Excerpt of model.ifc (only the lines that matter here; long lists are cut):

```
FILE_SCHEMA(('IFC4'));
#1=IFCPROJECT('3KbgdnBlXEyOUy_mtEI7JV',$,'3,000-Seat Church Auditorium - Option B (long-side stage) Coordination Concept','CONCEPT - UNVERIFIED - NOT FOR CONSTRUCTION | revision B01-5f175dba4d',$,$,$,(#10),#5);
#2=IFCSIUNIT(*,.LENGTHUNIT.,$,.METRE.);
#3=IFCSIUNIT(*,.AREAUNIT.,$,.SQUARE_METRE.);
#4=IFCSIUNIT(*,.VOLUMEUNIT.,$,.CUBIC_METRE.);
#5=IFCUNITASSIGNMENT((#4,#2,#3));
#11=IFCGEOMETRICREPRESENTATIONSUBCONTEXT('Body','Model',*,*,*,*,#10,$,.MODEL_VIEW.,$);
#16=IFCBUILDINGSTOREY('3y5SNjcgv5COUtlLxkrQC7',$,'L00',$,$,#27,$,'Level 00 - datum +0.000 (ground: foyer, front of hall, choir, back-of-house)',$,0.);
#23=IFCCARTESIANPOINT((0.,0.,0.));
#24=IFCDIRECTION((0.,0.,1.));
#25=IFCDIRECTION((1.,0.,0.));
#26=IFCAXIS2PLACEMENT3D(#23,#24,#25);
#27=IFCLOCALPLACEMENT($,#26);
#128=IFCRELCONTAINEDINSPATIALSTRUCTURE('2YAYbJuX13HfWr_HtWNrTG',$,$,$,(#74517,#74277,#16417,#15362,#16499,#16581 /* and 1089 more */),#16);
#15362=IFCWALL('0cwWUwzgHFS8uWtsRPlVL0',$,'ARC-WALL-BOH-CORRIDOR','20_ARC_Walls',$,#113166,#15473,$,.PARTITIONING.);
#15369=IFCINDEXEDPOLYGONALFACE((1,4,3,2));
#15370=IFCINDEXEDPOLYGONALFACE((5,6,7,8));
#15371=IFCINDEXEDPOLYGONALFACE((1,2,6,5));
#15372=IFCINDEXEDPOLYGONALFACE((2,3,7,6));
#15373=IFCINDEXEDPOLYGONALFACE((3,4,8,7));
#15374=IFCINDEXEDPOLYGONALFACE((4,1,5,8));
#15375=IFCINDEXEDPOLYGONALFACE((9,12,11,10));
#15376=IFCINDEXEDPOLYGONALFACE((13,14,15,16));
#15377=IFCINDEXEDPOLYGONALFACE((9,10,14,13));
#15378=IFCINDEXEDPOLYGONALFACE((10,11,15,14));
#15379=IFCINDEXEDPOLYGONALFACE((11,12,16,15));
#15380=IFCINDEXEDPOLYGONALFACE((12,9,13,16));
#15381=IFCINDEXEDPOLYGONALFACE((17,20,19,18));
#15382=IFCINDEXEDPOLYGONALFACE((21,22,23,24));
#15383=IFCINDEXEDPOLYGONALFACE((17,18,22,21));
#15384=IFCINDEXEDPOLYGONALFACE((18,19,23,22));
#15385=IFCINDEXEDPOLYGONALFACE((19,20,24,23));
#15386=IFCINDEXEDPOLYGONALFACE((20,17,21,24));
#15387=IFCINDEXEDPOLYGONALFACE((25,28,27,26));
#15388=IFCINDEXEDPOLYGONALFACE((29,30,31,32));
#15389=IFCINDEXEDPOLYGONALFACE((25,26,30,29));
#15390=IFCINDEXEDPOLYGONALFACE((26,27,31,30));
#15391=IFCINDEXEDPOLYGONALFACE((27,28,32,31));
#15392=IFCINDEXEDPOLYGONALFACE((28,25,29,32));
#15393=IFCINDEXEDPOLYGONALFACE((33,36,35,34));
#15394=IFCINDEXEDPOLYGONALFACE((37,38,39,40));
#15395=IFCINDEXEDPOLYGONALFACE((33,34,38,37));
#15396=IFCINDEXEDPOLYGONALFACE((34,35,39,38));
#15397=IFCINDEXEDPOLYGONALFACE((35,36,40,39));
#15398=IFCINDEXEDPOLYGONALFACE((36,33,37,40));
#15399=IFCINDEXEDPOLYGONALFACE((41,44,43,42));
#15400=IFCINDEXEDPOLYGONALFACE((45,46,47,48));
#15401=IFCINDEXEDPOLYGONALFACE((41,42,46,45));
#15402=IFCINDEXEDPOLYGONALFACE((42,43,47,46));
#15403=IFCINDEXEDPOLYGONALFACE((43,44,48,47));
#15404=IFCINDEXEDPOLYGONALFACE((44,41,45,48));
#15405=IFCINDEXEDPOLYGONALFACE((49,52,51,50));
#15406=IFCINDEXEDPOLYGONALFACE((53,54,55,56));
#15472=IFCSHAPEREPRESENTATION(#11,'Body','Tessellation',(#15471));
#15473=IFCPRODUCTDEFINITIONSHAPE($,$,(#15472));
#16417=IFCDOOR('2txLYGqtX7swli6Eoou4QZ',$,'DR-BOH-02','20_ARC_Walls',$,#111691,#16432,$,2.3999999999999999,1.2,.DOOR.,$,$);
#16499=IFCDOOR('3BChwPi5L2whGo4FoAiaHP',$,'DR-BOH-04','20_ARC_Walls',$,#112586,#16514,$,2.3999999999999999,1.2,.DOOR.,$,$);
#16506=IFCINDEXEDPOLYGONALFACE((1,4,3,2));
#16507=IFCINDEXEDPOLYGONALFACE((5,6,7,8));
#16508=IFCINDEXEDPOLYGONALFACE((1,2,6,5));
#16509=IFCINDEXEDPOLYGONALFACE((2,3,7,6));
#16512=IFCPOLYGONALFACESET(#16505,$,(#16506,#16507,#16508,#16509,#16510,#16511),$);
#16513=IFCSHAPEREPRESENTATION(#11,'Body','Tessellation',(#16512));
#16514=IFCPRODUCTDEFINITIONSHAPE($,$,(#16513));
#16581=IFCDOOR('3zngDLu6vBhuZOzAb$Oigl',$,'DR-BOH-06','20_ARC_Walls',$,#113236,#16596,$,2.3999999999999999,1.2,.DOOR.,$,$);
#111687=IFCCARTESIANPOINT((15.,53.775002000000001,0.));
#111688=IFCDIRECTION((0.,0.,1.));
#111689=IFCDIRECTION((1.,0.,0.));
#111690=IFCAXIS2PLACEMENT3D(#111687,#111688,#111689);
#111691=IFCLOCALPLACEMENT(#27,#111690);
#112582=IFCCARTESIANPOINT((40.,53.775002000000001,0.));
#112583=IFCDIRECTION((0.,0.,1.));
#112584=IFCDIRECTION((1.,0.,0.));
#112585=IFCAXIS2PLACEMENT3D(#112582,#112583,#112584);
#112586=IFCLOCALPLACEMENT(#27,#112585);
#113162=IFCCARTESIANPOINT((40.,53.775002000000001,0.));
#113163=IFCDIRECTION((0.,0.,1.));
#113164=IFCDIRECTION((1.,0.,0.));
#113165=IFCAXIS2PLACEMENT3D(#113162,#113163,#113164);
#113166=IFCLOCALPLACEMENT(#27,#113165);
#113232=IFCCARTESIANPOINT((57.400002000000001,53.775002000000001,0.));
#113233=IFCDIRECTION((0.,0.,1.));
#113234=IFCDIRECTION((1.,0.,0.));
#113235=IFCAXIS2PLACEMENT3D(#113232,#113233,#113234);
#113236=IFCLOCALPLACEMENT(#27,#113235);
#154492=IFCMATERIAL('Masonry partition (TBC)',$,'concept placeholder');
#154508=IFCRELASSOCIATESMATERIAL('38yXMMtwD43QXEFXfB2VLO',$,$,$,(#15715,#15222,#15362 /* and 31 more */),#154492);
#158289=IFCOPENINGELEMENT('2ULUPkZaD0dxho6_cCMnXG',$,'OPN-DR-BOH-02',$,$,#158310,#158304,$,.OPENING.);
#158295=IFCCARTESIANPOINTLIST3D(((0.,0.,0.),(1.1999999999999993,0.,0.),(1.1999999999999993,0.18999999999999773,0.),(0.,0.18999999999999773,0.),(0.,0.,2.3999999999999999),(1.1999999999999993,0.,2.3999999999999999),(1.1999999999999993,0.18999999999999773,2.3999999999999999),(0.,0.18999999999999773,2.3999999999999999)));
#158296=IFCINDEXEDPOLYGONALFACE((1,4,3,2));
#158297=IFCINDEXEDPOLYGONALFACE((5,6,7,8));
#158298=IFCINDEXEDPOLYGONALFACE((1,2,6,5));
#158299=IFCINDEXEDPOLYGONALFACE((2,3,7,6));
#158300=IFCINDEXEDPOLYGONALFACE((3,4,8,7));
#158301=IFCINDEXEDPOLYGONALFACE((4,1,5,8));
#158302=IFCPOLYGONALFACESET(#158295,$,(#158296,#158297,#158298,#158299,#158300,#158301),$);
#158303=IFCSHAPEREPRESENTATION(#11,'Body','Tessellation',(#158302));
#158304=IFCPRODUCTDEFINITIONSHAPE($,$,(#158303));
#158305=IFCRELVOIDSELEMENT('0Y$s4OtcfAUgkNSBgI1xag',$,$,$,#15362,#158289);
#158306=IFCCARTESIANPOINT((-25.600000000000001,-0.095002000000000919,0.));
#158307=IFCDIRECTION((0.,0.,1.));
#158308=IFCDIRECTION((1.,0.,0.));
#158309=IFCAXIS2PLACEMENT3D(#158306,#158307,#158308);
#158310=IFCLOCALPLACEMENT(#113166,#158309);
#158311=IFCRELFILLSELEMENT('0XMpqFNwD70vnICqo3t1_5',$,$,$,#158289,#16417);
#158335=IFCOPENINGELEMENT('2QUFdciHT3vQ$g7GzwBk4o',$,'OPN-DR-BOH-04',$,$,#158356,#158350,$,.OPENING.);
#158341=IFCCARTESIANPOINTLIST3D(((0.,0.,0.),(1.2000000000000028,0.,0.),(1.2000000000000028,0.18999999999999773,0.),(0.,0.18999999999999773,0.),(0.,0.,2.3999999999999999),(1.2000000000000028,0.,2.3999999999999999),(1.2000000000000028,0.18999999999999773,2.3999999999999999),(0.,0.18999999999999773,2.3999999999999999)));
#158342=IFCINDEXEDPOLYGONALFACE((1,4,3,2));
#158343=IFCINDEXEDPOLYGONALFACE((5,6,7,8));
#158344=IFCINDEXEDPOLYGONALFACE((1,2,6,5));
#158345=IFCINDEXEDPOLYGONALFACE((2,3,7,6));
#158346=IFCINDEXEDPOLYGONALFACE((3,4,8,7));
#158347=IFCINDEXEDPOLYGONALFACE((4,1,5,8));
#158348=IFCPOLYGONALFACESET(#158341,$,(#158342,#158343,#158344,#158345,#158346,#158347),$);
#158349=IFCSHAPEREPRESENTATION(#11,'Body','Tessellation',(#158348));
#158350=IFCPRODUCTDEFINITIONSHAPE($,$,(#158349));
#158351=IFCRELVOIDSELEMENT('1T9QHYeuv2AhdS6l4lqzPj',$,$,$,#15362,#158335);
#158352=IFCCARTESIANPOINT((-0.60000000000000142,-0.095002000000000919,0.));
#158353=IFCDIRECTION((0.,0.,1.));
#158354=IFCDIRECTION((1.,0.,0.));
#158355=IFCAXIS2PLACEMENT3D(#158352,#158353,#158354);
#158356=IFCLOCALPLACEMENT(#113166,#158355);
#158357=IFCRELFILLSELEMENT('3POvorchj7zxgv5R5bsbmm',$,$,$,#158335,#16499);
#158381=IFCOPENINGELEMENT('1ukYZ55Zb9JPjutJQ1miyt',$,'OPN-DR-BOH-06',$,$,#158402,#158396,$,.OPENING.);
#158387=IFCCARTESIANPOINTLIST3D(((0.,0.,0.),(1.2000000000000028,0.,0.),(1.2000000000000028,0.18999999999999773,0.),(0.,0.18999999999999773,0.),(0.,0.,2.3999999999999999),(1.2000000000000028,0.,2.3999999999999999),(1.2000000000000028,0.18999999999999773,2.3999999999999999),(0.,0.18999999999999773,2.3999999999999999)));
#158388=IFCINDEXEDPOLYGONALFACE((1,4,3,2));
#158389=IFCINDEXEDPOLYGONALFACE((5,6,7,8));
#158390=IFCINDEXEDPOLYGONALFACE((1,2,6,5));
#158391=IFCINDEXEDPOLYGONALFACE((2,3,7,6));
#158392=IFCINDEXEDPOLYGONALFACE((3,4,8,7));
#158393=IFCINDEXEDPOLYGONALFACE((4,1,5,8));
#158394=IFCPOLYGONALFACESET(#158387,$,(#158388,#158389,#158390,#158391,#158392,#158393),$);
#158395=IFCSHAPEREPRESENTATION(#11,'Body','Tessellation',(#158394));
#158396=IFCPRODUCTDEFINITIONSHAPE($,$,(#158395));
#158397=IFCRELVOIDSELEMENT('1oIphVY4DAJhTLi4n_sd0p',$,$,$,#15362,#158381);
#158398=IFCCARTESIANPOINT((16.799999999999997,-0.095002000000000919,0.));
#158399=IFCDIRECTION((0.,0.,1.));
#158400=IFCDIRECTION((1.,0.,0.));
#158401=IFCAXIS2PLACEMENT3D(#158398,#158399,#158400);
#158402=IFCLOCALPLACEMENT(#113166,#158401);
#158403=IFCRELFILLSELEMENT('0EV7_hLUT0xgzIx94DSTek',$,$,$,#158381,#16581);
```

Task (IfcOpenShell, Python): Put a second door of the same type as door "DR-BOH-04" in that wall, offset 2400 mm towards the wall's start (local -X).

```python
import ifcopenshell
import ifcopenshell.api.feature
import ifcopenshell.api.geometry
import ifcopenshell.api.root
import ifcopenshell.geom
import ifcopenshell.util.element
import ifcopenshell.util.placement
import ifcopenshell.util.shape
import ifcopenshell.util.unit

model = ifcopenshell.open("model.ifc")
unit_scale = ifcopenshell.util.unit.calculate_unit_scale(model)
settings = ifcopenshell.geom.settings()


def volume(element):
    """Net volume in cubic metres, openings subtracted."""
    shape = ifcopenshell.geom.create_shape(settings, element)
    return ifcopenshell.util.shape.get_volume(shape.geometry)


door = model.by_guid("3BChwPi5L2whGo4FoAiaHP")
opening = door.FillsVoids[0].RelatingOpeningElement
wall = opening.VoidsElements[0].RelatingBuildingElement
before = volume(wall)
shift = ifcopenshell.util.placement.get_local_placement(wall.ObjectPlacement)[:3, 0] * -2.4 / unit_scale

# copy_class copies the void relationship, type, container and properties, but no geometry.
new_opening = ifcopenshell.api.root.copy_class(model, product=opening)
new_opening.Representation = ifcopenshell.util.element.copy_deep(
    model, opening.Representation, exclude=["IfcGeometricRepresentationContext", "IfcRepresentationMap"]
)
new_door = ifcopenshell.api.root.copy_class(model, product=door)
new_door.Representation = ifcopenshell.util.element.copy_deep(
    model, door.Representation, exclude=["IfcGeometricRepresentationContext", "IfcRepresentationMap"]
)
ifcopenshell.api.feature.add_filling(model, opening=new_opening, element=new_door)

for old, new in ((opening, new_opening), (door, new_door)):
    matrix = ifcopenshell.util.placement.get_local_placement(old.ObjectPlacement)
    matrix[:3, 3] += shift
    ifcopenshell.api.geometry.edit_object_placement(model, product=new, matrix=matrix, is_si=False)

after = volume(wall)

print(f"wall volume {before:.3f} -> {after:.3f} m3")

model.write("model_updated.ifc")
```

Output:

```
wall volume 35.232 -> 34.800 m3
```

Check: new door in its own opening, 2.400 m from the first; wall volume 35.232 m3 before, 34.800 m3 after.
